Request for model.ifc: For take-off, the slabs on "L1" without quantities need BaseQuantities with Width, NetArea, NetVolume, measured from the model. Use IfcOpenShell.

First a look at what the model holds.

```python
import ifcopenshell
import ifcopenshell.util.element
import ifcopenshell.util.unit

model = ifcopenshell.open("model.ifc")
print(model.schema)
for unit_type in ("LENGTHUNIT", "AREAUNIT", "VOLUMEUNIT"):
    print(unit_type, ifcopenshell.util.unit.calculate_unit_scale(model, unit_type))
storey = next(s for s in model.by_type("IfcBuildingStorey") if s.Name == "L1")
slabs = [e for e in ifcopenshell.util.element.get_decomposition(storey) if e.is_a("IfcSlab")]
for e in sorted(slabs, key=lambda e: e.id()):
    print(e.id(), e.is_a(), e.Name, list(ifcopenshell.util.element.get_psets(e, qtos_only=True)), sep=" | ")
```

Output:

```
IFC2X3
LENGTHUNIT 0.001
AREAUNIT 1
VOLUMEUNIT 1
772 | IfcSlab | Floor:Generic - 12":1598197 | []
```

```python
import ifcopenshell
import ifcopenshell.api.pset
import ifcopenshell.geom
import ifcopenshell.util.element
import ifcopenshell.util.shape
import ifcopenshell.util.unit

model = ifcopenshell.open("model.ifc")
unit_scale = ifcopenshell.util.unit.calculate_unit_scale(model)
area_scale = ifcopenshell.util.unit.calculate_unit_scale(model, "AREAUNIT")
volume_scale = ifcopenshell.util.unit.calculate_unit_scale(model, "VOLUMEUNIT")
settings = ifcopenshell.geom.settings()

storey = next(s for s in model.by_type("IfcBuildingStorey") if s.Name == "L1")
slabs = [e for e in ifcopenshell.util.element.get_decomposition(storey) if e.is_a("IfcSlab")]

for e in sorted(slabs, key=lambda e: e.id()):
    if ifcopenshell.util.element.get_psets(e, qtos_only=True, should_inherit=False):
        continue
    # Geometry comes back in metres, in the element's own axes.
    shape = ifcopenshell.geom.create_shape(settings, e)
    values = {
        "Width": ifcopenshell.util.shape.get_z(shape.geometry) / unit_scale,
        "NetArea": ifcopenshell.util.shape.get_footprint_area(shape.geometry) / area_scale,
        "NetVolume": ifcopenshell.util.shape.get_volume(shape.geometry) / volume_scale,
    }
    qto = ifcopenshell.api.pset.add_qto(model, product=e, name="BaseQuantities")
    ifcopenshell.api.pset.edit_qto(model, qto=qto, properties=values)
    print(e.id(), {k: round(v, 3) for k, v in values.items()})

model.write("model-out.ifc")
```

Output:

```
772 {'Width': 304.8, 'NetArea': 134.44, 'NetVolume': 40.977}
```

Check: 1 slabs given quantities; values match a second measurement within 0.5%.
